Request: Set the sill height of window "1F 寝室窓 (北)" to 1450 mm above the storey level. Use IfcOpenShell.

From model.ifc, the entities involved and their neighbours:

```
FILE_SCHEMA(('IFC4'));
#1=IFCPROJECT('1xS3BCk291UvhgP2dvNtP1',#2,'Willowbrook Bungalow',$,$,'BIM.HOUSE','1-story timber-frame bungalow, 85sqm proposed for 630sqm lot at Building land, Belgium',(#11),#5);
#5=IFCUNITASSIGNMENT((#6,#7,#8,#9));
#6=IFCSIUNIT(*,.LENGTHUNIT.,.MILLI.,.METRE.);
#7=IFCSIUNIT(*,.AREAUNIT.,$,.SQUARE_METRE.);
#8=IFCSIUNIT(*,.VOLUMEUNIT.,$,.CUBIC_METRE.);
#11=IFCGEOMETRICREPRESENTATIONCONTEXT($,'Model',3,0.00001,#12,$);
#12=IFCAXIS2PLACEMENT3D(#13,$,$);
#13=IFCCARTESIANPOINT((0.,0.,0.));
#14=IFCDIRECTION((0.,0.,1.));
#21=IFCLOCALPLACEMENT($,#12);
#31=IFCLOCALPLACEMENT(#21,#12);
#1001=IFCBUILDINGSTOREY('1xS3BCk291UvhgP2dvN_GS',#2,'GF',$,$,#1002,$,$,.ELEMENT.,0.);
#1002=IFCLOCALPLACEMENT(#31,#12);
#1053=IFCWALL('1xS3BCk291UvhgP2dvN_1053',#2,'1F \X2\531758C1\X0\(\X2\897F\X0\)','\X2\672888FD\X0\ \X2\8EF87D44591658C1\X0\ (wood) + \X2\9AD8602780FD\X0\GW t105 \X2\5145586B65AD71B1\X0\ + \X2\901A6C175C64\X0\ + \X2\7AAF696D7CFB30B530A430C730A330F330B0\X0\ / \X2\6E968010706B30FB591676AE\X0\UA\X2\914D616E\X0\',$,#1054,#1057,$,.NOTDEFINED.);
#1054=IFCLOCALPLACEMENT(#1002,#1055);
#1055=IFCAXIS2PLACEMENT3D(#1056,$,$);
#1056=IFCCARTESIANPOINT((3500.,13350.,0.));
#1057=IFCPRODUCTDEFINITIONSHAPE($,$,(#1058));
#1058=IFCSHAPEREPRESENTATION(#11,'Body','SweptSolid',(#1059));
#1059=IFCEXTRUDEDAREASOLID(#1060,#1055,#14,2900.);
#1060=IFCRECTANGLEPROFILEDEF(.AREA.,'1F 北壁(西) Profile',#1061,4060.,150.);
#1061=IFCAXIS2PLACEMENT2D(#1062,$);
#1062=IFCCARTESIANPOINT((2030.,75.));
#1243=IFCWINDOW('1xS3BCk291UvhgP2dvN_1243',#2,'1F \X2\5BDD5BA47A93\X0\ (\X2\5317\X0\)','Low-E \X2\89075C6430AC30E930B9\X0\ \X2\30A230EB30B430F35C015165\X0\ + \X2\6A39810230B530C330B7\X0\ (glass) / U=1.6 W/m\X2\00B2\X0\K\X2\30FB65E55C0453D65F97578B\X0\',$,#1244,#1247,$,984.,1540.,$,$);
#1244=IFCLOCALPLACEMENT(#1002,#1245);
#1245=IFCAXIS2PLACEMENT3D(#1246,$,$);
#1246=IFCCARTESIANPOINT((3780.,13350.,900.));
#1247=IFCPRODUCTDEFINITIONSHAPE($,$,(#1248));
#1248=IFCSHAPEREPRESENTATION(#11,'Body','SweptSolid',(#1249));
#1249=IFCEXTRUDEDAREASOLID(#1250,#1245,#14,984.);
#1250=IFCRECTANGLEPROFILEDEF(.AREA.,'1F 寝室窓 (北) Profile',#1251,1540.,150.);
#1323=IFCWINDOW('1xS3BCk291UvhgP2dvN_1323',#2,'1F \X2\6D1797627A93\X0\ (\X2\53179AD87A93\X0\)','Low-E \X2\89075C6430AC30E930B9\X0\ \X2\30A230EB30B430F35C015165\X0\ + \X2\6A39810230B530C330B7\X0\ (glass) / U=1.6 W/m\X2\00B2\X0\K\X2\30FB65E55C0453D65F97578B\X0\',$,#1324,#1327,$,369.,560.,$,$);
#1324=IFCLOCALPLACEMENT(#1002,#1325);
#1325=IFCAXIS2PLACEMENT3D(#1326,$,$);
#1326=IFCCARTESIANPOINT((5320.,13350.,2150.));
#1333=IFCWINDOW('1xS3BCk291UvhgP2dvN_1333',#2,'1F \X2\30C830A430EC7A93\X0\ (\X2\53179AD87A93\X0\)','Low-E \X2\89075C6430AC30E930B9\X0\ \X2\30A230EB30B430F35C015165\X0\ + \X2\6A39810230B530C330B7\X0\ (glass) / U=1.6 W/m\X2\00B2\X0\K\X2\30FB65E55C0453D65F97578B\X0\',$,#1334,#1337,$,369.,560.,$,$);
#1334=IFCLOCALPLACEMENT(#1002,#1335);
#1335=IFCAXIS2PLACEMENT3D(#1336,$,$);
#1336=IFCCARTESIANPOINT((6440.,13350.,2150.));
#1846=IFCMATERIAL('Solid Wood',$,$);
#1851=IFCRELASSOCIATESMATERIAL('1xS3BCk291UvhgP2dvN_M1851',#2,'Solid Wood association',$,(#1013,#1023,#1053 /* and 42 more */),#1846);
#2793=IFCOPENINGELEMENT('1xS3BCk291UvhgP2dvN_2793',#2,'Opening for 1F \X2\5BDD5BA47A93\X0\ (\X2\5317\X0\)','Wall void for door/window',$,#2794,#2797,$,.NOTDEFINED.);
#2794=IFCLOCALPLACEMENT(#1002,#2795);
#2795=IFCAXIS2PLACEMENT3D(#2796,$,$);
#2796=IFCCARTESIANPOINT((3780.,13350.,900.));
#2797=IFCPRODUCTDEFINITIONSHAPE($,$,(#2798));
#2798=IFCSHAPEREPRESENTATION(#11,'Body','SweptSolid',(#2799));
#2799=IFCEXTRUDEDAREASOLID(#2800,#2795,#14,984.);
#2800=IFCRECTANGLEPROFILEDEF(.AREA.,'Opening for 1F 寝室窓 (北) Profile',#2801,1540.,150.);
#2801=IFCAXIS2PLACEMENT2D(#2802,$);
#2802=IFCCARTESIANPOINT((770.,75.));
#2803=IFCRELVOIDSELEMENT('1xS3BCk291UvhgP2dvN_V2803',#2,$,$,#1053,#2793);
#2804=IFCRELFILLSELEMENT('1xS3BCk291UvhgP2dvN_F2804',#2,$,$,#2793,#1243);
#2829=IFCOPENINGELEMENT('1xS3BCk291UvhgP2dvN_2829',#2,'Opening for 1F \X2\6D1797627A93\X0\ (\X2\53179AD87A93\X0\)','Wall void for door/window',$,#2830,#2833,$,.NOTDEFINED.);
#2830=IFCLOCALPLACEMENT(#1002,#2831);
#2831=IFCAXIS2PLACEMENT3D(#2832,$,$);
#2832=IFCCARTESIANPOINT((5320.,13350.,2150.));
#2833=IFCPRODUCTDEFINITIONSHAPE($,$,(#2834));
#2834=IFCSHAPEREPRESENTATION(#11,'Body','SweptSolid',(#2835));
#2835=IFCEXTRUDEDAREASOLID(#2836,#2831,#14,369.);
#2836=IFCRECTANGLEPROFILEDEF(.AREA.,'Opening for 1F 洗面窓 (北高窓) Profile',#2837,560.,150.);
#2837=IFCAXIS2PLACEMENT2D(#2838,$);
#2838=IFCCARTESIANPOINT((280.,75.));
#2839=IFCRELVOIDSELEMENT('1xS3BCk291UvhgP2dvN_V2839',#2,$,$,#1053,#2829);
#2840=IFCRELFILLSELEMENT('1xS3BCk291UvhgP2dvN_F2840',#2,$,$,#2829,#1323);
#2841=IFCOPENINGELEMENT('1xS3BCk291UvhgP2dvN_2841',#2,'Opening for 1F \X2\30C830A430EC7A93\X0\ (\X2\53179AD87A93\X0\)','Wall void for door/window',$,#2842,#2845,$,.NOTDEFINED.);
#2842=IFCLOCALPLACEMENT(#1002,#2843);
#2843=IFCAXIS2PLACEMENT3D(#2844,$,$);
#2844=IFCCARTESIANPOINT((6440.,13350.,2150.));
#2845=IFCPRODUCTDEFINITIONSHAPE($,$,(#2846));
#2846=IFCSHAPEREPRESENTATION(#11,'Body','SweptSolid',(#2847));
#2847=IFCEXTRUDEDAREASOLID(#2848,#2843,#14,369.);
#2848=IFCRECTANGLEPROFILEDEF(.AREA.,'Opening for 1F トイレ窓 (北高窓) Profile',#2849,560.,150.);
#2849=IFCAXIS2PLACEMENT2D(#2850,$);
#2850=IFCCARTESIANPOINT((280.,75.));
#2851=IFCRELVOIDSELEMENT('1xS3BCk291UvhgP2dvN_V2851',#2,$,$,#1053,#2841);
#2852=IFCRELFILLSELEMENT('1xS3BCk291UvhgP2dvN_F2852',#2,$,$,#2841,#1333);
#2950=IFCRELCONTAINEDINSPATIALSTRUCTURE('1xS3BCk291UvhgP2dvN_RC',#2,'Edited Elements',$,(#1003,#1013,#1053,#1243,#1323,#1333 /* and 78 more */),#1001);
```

```python
import numpy as np
import ifcopenshell
import ifcopenshell.api.geometry
import ifcopenshell.geom
import ifcopenshell.util.element
import ifcopenshell.util.placement
import ifcopenshell.util.shape
import ifcopenshell.util.unit

model = ifcopenshell.open("model.ifc")
unit_scale = ifcopenshell.util.unit.calculate_unit_scale(model)

window = model.by_guid("1xS3BCk291UvhgP2dvN_1243")
opening = window.FillsVoids[0].RelatingOpeningElement
storey = ifcopenshell.util.element.get_container(window, ifc_class="IfcBuildingStorey")
level = ifcopenshell.util.placement.get_local_placement(storey.ObjectPlacement)[2, 3]

# The opening's origin need not be at the sill, so measure its lowest point.
shape = ifcopenshell.geom.create_shape(ifcopenshell.geom.settings(), opening)
bottom = ifcopenshell.util.shape.get_shape_bottom_elevation(shape, shape.geometry) / unit_scale
dz = level + 1.45 / unit_scale - bottom

shift = np.array([0.0, 0.0, dz])
# The window is not placed relative to its opening, so move both.
for product in (opening, window):
    matrix = ifcopenshell.util.placement.get_local_placement(product.ObjectPlacement)
    matrix[:3, 3] += shift
    ifcopenshell.api.geometry.edit_object_placement(model, product=product, matrix=matrix, is_si=False)

print(f"moved by {dz * unit_scale:+.3f} m")

model.write("model_edited.ifc")
```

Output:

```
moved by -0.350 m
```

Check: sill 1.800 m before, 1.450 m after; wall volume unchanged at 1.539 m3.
